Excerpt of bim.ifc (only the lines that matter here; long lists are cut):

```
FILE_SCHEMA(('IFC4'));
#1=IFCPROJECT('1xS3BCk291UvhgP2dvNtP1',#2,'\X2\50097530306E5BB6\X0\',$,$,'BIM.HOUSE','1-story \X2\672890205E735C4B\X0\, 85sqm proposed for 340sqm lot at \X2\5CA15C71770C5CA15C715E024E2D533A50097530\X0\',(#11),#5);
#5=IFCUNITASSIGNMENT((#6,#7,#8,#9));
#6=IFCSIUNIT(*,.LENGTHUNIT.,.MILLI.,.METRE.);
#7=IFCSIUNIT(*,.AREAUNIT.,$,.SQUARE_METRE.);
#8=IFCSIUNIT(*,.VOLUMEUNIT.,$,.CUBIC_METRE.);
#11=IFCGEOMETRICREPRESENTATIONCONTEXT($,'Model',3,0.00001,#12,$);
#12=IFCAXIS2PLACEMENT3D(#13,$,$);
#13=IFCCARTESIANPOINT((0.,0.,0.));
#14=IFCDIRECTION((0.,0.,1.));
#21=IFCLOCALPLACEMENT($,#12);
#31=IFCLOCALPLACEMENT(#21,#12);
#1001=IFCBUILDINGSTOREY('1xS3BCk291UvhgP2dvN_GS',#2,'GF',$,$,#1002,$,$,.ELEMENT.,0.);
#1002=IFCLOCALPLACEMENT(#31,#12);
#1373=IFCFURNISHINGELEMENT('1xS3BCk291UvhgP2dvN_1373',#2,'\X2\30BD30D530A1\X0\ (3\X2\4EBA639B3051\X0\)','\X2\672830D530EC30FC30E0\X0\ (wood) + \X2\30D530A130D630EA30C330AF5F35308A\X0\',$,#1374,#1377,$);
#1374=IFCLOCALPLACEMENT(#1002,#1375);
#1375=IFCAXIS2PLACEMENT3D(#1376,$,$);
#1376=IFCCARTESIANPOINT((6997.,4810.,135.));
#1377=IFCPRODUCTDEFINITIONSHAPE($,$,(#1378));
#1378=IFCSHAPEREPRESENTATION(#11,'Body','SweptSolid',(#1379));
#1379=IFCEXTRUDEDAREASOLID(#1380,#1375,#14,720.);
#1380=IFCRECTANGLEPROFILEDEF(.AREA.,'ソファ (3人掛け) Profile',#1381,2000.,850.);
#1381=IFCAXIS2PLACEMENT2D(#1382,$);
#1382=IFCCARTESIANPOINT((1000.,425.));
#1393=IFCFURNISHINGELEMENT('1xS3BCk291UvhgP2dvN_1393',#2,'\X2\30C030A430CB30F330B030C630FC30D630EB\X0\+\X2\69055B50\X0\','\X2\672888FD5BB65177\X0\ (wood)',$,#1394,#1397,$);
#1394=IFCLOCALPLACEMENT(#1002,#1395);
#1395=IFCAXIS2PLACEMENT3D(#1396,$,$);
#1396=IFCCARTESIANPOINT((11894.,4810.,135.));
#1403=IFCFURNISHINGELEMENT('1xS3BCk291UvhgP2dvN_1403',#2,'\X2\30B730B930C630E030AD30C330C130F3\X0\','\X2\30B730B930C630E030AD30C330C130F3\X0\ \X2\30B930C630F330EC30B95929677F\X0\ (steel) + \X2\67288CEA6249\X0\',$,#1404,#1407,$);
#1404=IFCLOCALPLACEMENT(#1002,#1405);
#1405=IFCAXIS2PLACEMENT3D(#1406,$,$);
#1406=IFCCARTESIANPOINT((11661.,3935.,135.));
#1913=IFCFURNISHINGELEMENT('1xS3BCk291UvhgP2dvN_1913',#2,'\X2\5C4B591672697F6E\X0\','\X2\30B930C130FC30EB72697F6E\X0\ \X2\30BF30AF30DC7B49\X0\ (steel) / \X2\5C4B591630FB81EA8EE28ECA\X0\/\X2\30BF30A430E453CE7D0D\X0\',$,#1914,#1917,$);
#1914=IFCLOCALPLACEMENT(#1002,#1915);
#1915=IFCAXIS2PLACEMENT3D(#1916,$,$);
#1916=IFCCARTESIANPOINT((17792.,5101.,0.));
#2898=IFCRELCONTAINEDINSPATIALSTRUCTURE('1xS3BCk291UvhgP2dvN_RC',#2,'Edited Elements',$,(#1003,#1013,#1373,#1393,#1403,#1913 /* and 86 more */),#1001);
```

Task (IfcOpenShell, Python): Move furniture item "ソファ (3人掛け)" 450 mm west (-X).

```python
import ifcopenshell
import ifcopenshell.api.geometry
import ifcopenshell.util.placement
import ifcopenshell.util.unit

model = ifcopenshell.open("bim.ifc")
unit_scale = ifcopenshell.util.unit.calculate_unit_scale(model)

item = model.by_guid("1xS3BCk291UvhgP2dvN_1373")
matrix = ifcopenshell.util.placement.get_local_placement(item.ObjectPlacement)
matrix[0, 3] -= 0.45 / unit_scale
ifcopenshell.api.geometry.edit_object_placement(model, product=item, matrix=matrix, is_si=False)

print(ifcopenshell.util.placement.get_local_placement(item.ObjectPlacement).round(3) + 0.0)

model.write("bim-out.ifc")
```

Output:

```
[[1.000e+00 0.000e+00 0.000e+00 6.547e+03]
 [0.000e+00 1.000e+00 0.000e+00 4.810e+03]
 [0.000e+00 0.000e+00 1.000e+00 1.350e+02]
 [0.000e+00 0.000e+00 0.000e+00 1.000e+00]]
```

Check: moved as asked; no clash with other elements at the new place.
